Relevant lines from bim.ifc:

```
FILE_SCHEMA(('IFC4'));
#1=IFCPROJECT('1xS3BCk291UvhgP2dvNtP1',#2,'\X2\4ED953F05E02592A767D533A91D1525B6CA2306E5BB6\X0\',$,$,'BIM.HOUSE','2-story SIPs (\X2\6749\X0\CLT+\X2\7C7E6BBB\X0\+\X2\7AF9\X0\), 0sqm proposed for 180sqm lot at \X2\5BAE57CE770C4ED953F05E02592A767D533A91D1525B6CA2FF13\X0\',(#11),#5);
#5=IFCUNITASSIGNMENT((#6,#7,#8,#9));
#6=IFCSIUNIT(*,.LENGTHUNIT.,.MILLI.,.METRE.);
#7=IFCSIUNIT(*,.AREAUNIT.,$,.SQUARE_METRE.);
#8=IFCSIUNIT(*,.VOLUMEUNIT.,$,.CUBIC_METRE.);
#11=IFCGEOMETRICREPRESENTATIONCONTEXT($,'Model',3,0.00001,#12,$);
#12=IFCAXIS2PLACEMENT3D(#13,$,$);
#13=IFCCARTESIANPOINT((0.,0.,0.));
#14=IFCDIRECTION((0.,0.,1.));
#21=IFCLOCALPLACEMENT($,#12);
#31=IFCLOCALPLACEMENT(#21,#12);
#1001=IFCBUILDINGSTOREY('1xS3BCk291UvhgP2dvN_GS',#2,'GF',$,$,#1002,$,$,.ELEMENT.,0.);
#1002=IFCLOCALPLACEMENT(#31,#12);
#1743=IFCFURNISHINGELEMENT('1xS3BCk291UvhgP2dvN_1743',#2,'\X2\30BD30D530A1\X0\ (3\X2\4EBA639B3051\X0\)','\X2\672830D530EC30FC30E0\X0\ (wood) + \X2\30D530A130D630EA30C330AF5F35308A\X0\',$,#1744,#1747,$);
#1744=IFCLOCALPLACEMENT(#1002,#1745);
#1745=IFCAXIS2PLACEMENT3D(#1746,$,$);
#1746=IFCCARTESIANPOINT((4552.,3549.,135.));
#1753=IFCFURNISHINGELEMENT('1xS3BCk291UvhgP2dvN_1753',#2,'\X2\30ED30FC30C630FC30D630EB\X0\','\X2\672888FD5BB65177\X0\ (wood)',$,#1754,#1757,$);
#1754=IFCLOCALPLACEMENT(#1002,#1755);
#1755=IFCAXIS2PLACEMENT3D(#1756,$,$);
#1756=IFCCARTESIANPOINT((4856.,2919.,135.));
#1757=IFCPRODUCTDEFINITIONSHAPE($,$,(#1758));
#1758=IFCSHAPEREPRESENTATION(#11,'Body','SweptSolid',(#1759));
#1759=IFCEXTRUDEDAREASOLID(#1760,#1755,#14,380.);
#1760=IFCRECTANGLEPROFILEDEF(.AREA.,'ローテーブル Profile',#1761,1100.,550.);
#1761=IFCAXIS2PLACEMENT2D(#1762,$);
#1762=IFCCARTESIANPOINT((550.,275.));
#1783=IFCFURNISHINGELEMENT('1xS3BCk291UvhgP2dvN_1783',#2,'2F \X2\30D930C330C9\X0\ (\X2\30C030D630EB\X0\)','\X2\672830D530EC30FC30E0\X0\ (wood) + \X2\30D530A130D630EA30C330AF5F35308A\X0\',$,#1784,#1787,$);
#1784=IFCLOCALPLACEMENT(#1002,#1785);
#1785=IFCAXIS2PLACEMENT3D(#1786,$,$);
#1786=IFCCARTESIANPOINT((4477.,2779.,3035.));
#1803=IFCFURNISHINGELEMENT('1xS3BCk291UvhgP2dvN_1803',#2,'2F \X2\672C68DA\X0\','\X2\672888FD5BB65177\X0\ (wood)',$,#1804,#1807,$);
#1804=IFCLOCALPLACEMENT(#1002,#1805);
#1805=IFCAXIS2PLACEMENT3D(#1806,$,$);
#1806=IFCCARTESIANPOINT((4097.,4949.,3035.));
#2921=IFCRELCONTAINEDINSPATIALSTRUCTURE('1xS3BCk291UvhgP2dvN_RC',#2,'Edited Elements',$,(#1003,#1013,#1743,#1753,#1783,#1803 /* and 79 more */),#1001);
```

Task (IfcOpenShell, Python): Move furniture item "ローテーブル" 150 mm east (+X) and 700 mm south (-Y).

```python
import ifcopenshell
import ifcopenshell.api.geometry
import ifcopenshell.util.placement

model = ifcopenshell.open("bim.ifc")

item = model.by_guid("1xS3BCk291UvhgP2dvN_1753")
matrix = ifcopenshell.util.placement.get_local_placement(item.ObjectPlacement)
matrix[0, 3] += 150.0
matrix[1, 3] -= 700.0
ifcopenshell.api.geometry.edit_object_placement(model, product=item, matrix=matrix, is_si=False)

print(ifcopenshell.util.placement.get_local_placement(item.ObjectPlacement).round(3) + 0.0)

model.write("bim_v2.ifc")
```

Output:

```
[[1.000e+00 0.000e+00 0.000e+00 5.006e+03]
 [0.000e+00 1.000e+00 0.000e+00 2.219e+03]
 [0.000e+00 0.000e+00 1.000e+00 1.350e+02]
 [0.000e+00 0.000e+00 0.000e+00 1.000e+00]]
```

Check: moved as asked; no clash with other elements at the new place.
